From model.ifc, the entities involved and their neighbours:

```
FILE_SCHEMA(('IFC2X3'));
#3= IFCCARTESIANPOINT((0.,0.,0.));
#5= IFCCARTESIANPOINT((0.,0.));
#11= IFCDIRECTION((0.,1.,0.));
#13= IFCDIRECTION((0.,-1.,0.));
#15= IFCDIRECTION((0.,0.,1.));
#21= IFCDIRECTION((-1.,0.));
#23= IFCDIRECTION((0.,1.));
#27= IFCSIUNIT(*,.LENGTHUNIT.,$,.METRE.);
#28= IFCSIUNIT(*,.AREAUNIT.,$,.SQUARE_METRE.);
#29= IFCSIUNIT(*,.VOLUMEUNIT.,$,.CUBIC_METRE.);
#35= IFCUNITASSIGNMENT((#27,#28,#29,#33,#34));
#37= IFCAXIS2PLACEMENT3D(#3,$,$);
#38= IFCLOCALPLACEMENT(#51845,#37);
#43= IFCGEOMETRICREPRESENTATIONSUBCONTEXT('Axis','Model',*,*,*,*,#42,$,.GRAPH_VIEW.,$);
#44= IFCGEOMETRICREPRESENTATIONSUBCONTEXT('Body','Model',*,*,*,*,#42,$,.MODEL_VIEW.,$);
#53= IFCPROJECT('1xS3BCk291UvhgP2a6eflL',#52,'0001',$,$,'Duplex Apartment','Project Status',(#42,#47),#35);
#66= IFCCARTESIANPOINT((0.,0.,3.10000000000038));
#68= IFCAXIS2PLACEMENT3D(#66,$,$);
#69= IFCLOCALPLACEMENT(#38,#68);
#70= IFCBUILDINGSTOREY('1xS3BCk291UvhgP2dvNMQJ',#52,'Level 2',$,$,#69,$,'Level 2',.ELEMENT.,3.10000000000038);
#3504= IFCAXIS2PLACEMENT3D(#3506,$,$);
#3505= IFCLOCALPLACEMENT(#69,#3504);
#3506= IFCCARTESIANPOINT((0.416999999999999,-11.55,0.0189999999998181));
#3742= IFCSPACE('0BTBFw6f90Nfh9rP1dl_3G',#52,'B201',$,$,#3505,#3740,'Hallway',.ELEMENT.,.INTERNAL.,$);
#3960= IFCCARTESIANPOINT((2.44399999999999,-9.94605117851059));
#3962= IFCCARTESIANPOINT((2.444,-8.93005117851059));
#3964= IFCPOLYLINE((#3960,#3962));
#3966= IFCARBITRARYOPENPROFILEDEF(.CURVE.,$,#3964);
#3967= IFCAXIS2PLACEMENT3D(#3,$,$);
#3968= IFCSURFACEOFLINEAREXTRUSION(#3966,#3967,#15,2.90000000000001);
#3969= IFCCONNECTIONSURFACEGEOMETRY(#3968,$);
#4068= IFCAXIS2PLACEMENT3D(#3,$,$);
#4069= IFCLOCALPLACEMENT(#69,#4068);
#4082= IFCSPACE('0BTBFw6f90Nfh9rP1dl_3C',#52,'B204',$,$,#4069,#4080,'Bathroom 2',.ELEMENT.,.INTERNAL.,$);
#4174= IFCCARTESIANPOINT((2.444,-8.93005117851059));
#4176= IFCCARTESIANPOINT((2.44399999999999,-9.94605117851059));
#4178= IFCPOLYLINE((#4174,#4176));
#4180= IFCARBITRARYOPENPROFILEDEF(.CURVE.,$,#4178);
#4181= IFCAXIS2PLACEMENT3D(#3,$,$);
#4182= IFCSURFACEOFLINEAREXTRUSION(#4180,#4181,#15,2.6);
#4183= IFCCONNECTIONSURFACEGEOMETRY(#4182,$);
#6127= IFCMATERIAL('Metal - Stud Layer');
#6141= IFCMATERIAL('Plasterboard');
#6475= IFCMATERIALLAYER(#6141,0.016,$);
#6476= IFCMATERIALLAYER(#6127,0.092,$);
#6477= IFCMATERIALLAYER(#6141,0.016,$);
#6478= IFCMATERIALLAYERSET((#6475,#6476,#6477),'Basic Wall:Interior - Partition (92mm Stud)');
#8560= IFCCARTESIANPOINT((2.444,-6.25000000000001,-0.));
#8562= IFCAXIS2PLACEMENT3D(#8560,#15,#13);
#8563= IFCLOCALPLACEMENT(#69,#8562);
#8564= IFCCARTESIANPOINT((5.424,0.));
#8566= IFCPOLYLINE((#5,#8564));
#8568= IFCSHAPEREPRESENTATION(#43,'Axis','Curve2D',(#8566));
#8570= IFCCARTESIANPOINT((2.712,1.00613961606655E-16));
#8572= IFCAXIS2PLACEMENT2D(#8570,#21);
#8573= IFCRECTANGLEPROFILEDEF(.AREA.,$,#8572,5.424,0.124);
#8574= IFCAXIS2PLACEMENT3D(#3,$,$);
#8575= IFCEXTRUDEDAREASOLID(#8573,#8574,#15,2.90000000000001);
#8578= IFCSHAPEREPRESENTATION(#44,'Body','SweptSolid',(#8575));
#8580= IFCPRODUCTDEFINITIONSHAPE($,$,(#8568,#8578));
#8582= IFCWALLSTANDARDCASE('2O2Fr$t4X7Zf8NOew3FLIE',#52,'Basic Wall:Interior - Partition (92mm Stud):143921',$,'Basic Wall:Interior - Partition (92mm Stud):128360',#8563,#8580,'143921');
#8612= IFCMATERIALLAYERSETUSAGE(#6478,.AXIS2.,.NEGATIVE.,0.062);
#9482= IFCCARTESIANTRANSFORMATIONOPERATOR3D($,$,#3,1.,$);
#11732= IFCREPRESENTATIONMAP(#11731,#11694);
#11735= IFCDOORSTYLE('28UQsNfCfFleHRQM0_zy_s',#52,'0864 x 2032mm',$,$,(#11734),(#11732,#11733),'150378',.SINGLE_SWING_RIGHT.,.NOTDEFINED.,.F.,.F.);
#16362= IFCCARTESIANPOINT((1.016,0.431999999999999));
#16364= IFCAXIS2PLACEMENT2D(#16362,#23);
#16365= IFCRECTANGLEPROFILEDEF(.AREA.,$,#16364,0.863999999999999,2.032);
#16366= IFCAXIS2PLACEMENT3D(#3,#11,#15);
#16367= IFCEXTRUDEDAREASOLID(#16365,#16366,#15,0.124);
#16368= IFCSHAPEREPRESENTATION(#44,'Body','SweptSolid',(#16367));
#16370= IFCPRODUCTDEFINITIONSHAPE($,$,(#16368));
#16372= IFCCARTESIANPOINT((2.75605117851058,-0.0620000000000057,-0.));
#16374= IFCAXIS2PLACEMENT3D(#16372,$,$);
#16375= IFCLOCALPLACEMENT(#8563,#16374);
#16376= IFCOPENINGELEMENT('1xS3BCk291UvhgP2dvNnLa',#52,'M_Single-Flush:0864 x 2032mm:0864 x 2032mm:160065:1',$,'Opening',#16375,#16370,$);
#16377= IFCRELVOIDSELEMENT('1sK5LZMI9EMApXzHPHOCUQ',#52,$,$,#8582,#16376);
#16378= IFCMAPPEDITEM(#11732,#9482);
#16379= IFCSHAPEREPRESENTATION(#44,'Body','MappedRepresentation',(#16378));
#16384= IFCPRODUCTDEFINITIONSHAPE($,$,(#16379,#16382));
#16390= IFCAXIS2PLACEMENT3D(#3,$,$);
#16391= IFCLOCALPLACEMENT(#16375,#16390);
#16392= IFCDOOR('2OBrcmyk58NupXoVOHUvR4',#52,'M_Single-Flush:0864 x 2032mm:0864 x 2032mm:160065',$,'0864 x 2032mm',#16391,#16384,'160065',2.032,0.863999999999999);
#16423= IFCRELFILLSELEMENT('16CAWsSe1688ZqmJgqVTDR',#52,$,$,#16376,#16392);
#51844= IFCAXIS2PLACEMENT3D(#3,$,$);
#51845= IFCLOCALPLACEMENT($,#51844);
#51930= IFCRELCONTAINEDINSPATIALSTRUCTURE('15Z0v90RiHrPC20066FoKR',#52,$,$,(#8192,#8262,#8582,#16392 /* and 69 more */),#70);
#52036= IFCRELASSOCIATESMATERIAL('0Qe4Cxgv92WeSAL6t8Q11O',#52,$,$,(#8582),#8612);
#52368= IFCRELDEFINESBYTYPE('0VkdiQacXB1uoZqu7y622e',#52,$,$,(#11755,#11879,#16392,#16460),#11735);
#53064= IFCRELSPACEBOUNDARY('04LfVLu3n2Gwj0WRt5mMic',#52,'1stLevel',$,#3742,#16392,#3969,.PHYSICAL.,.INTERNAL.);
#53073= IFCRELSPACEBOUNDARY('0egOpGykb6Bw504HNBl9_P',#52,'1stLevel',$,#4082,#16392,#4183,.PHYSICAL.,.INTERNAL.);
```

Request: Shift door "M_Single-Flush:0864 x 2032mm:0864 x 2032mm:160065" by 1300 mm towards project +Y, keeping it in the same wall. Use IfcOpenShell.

```python
import numpy as np
import ifcopenshell
import ifcopenshell.api.geometry
import ifcopenshell.util.placement
import ifcopenshell.util.unit

model = ifcopenshell.open("model.ifc")
unit_scale = ifcopenshell.util.unit.calculate_unit_scale(model)

door = model.by_guid("2OBrcmyk58NupXoVOHUvR4")
opening = door.FillsVoids[0].RelatingOpeningElement
wall = opening.VoidsElements[0].RelatingBuildingElement

wall_matrix = ifcopenshell.util.placement.get_local_placement(wall.ObjectPlacement)
shift = wall_matrix[:3, 0] * -1.3 / unit_scale
before = ifcopenshell.util.placement.get_local_placement(door.ObjectPlacement)[:3, 3].copy()

# The door is placed relative to its opening, so it follows when the opening moves.
matrix = ifcopenshell.util.placement.get_local_placement(opening.ObjectPlacement)
matrix[:3, 3] += shift
ifcopenshell.api.geometry.edit_object_placement(
    model, product=opening, matrix=matrix, is_si=False, should_transform_children=True
)

# Space boundary surfaces are stored in each space's coordinates; move them too.
for rel in door.ProvidesBoundaries:
    if not rel.ConnectionGeometry:
        continue
    surface = rel.ConnectionGeometry.SurfaceOnRelatingElement
    space_matrix = ifcopenshell.util.placement.get_local_placement(rel.RelatingSpace.ObjectPlacement)
    point = np.array(surface.Position.Location.Coordinates) + space_matrix[:3, :3].T @ shift
    surface.Position = model.createIfcAxis2Placement3D(
        model.createIfcCartesianPoint(point.tolist()), surface.Position.Axis, surface.Position.RefDirection
    )

after = ifcopenshell.util.placement.get_local_placement(door.ObjectPlacement)[:3, 3]
print("door moved by", (after - before).round(3) + 0.0)

model.write("model_edited.ifc")
```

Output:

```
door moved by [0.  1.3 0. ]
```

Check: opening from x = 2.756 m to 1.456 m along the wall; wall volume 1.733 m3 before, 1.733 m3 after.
